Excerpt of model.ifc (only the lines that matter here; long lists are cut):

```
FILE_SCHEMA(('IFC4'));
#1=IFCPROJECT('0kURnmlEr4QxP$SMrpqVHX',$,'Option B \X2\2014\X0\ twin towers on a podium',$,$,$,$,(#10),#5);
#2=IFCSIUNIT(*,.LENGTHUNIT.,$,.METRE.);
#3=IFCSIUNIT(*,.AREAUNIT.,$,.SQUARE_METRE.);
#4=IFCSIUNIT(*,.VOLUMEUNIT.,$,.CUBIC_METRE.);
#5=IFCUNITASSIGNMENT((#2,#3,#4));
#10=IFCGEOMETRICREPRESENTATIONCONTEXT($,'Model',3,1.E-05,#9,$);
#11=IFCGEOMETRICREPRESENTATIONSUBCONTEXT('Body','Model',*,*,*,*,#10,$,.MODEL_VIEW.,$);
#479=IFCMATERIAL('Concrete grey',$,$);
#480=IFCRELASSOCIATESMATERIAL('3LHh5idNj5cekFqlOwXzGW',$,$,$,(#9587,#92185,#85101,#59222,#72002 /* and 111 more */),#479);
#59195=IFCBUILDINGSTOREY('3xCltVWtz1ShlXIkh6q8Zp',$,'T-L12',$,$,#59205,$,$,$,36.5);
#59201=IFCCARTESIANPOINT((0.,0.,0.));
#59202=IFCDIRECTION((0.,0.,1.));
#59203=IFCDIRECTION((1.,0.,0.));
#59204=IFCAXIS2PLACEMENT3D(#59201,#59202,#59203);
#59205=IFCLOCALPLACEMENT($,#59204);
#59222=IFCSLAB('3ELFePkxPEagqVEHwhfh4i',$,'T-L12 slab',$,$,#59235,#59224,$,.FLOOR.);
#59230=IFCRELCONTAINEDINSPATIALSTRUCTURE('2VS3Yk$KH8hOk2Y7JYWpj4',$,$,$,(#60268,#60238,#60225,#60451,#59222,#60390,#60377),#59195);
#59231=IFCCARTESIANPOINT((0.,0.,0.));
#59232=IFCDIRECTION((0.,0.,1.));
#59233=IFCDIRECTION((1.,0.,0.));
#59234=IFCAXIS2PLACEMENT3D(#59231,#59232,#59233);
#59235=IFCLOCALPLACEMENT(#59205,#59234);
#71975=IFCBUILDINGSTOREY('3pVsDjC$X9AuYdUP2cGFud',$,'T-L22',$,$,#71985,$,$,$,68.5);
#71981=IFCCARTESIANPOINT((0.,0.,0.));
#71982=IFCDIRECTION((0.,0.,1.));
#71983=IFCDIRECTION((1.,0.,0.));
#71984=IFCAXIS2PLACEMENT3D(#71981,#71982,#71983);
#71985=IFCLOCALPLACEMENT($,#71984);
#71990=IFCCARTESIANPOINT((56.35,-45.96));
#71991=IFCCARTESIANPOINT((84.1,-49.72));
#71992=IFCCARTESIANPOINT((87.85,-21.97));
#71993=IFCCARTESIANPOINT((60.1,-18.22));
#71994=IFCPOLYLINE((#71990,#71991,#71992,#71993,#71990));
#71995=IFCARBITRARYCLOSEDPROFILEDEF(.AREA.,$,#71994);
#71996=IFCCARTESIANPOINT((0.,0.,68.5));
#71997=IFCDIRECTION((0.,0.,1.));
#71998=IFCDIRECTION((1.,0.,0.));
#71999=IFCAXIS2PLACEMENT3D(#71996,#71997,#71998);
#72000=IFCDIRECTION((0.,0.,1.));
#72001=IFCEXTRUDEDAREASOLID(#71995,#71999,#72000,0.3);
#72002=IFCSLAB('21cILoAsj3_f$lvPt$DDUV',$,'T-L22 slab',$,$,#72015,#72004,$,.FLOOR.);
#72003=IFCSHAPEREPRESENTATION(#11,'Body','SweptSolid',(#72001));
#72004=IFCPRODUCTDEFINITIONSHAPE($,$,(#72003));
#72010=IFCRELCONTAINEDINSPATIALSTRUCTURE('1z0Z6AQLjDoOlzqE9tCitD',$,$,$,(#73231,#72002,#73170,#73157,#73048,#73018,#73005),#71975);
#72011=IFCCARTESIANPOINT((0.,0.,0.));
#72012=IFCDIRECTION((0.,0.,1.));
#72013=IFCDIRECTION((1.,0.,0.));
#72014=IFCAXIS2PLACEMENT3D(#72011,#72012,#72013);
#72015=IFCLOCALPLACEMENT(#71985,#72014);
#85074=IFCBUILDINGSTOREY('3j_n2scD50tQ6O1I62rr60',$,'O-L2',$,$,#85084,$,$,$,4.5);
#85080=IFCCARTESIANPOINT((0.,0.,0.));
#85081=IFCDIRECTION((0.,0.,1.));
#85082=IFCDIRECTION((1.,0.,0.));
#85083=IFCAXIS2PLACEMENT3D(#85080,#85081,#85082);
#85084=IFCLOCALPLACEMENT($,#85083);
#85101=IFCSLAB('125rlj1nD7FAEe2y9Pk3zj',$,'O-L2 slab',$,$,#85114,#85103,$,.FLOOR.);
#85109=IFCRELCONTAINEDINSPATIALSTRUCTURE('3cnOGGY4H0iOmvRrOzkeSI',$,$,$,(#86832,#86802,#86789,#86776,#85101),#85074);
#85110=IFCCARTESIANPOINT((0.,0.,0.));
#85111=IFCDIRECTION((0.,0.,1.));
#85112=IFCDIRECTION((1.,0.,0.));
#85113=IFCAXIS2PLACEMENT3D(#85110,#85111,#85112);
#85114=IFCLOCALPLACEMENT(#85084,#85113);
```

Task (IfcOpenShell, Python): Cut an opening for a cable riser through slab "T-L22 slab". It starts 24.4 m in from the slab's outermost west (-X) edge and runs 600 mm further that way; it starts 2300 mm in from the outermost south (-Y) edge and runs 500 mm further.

```python
import numpy as np
import ifcopenshell
import ifcopenshell.api.feature
import ifcopenshell.api.geometry
import ifcopenshell.api.root
import ifcopenshell.geom
import ifcopenshell.util.placement
import ifcopenshell.util.representation
import ifcopenshell.util.shape
import ifcopenshell.util.unit

model = ifcopenshell.open("model.ifc")
unit_scale = ifcopenshell.util.unit.calculate_unit_scale(model)
settings = ifcopenshell.geom.settings()


def volume(element):
    """Net volume in cubic metres, openings subtracted."""
    shape = ifcopenshell.geom.create_shape(settings, element)
    return ifcopenshell.util.shape.get_volume(shape.geometry)


slab = model.by_guid("21cILoAsj3_f$lvPt$DDUV")
before = volume(slab)

# Extent in the slab's own axes, in metres. The edges named are its -X and -Y sides.
slab_shape = ifcopenshell.geom.create_shape(settings, slab)
vertices = ifcopenshell.util.shape.get_vertices(slab_shape.geometry)
x_min, y_min, bottom = vertices.min(axis=0)
top = vertices[:, 2].max()

opening = ifcopenshell.api.root.create_entity(model, ifc_class="IfcOpeningElement", name="Cable riser opening", predefined_type="OPENING")
context = ifcopenshell.util.representation.get_context(model, "Model", "Body", "MODEL_VIEW")
width, depth = 0.6, 0.5
outline = [(0.0, 0.0), (width, 0.0), (width, depth), (0.0, depth), (0.0, 0.0)]
# Overshoot both faces by 50 mm so the cut is clean.
shape = ifcopenshell.api.geometry.add_slab_representation(
    model, context=context, depth=top - bottom + 0.1, polyline=outline
)
ifcopenshell.api.geometry.assign_representation(model, product=opening, representation=shape)

matrix = ifcopenshell.util.placement.get_local_placement(slab.ObjectPlacement)
matrix[:, 3] = matrix @ np.append(np.array([x_min + 24.4, y_min + 2.3, bottom - 0.05]) / unit_scale, 1.0)
ifcopenshell.api.geometry.edit_object_placement(model, product=opening, matrix=matrix, is_si=False)
ifcopenshell.api.feature.add_feature(model, feature=opening, element=slab)

after = volume(slab)

print(f"slab volume {before:.3f} -> {after:.3f} m3")

model.write("model_edited.ifc")
```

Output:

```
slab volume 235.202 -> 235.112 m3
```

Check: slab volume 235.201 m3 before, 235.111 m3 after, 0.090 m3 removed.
